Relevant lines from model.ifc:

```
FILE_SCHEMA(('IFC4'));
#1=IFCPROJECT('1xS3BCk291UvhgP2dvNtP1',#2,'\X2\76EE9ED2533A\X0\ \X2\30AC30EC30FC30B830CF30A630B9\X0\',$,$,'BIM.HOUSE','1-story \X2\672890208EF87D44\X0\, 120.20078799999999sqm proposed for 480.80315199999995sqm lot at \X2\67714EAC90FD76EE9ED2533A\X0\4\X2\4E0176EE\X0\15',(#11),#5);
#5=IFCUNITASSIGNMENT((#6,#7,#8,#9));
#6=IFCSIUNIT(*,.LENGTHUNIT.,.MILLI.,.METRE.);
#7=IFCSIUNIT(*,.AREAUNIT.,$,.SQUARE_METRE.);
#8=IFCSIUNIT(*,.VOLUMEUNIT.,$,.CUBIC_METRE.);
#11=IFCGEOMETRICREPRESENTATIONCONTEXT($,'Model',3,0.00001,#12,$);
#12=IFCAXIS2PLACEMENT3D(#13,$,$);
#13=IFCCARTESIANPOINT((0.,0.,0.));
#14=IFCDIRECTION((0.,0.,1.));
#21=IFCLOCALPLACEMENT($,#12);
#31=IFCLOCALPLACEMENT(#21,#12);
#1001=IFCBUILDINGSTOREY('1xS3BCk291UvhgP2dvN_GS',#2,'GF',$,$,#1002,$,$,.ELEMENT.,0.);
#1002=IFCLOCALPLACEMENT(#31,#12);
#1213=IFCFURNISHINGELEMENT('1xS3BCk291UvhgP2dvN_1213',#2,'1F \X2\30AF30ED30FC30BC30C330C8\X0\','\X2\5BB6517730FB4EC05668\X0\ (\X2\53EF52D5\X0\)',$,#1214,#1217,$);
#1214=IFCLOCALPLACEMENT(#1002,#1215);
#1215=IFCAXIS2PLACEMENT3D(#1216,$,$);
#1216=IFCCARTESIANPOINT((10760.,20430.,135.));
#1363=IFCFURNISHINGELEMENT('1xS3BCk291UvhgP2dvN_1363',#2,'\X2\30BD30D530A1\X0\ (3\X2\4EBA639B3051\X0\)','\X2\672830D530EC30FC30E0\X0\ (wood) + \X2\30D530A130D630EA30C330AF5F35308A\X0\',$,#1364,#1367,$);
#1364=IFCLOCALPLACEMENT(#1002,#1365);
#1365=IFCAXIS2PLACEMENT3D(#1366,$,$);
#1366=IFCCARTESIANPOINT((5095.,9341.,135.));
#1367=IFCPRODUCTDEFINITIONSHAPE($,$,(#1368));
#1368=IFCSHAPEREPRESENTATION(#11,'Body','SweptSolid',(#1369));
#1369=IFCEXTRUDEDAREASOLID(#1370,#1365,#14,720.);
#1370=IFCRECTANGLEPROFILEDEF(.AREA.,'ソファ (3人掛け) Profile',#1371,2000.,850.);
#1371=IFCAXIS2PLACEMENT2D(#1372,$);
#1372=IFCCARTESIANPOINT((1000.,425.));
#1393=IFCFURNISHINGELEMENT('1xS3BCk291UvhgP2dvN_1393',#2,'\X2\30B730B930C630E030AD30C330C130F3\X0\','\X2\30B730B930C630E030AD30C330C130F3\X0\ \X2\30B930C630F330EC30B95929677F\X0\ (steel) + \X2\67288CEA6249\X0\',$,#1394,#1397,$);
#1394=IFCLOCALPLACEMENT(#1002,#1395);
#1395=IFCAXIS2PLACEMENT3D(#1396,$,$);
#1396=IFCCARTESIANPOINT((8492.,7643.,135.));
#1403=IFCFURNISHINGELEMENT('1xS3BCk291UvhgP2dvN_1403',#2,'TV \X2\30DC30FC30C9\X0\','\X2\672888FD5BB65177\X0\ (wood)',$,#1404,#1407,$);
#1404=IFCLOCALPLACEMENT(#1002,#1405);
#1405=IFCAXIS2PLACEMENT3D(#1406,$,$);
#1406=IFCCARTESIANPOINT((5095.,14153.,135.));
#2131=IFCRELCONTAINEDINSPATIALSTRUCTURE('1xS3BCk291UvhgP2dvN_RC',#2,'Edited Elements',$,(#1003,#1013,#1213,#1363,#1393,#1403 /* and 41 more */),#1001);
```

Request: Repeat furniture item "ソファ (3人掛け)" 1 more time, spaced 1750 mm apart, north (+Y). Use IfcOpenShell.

```python
import numpy as np
import ifcopenshell
import ifcopenshell.api.geometry
import ifcopenshell.api.root
import ifcopenshell.util.element
import ifcopenshell.util.placement

model = ifcopenshell.open("model.ifc")


def reuse_history(source, copy):
    """copy_class also copies each property set's owner history, people and application; keep the originals."""
    for rel in copy.IsDefinedBy:
        if rel.is_a("IfcRelDefinesByProperties") and (history := rel.RelatingPropertyDefinition.OwnerHistory):
            rel.RelatingPropertyDefinition.OwnerHistory = source.OwnerHistory
            ifcopenshell.util.element.remove_deep2(model, history)


source = model.by_guid("1xS3BCk291UvhgP2dvN_1363")
base = ifcopenshell.util.placement.get_local_placement(source.ObjectPlacement)
step = np.array([0.0, 1.0, 0.0]) * 1750.0

for i in range(1, 2):
    copy = ifcopenshell.api.root.copy_class(model, product=source)
    copy.Representation = ifcopenshell.util.element.copy_deep(
        model, source.Representation, exclude=["IfcGeometricRepresentationContext", "IfcRepresentationMap"]
    )
    reuse_history(source, copy)
    matrix = base.copy()
    matrix[:3, 3] += i * step
    print("added at", matrix[:3, 3].round(3) + 0.0)
    ifcopenshell.api.geometry.edit_object_placement(model, product=copy, matrix=matrix, is_si=False)

model.write("model-out.ifc")
```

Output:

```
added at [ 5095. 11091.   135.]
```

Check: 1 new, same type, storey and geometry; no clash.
